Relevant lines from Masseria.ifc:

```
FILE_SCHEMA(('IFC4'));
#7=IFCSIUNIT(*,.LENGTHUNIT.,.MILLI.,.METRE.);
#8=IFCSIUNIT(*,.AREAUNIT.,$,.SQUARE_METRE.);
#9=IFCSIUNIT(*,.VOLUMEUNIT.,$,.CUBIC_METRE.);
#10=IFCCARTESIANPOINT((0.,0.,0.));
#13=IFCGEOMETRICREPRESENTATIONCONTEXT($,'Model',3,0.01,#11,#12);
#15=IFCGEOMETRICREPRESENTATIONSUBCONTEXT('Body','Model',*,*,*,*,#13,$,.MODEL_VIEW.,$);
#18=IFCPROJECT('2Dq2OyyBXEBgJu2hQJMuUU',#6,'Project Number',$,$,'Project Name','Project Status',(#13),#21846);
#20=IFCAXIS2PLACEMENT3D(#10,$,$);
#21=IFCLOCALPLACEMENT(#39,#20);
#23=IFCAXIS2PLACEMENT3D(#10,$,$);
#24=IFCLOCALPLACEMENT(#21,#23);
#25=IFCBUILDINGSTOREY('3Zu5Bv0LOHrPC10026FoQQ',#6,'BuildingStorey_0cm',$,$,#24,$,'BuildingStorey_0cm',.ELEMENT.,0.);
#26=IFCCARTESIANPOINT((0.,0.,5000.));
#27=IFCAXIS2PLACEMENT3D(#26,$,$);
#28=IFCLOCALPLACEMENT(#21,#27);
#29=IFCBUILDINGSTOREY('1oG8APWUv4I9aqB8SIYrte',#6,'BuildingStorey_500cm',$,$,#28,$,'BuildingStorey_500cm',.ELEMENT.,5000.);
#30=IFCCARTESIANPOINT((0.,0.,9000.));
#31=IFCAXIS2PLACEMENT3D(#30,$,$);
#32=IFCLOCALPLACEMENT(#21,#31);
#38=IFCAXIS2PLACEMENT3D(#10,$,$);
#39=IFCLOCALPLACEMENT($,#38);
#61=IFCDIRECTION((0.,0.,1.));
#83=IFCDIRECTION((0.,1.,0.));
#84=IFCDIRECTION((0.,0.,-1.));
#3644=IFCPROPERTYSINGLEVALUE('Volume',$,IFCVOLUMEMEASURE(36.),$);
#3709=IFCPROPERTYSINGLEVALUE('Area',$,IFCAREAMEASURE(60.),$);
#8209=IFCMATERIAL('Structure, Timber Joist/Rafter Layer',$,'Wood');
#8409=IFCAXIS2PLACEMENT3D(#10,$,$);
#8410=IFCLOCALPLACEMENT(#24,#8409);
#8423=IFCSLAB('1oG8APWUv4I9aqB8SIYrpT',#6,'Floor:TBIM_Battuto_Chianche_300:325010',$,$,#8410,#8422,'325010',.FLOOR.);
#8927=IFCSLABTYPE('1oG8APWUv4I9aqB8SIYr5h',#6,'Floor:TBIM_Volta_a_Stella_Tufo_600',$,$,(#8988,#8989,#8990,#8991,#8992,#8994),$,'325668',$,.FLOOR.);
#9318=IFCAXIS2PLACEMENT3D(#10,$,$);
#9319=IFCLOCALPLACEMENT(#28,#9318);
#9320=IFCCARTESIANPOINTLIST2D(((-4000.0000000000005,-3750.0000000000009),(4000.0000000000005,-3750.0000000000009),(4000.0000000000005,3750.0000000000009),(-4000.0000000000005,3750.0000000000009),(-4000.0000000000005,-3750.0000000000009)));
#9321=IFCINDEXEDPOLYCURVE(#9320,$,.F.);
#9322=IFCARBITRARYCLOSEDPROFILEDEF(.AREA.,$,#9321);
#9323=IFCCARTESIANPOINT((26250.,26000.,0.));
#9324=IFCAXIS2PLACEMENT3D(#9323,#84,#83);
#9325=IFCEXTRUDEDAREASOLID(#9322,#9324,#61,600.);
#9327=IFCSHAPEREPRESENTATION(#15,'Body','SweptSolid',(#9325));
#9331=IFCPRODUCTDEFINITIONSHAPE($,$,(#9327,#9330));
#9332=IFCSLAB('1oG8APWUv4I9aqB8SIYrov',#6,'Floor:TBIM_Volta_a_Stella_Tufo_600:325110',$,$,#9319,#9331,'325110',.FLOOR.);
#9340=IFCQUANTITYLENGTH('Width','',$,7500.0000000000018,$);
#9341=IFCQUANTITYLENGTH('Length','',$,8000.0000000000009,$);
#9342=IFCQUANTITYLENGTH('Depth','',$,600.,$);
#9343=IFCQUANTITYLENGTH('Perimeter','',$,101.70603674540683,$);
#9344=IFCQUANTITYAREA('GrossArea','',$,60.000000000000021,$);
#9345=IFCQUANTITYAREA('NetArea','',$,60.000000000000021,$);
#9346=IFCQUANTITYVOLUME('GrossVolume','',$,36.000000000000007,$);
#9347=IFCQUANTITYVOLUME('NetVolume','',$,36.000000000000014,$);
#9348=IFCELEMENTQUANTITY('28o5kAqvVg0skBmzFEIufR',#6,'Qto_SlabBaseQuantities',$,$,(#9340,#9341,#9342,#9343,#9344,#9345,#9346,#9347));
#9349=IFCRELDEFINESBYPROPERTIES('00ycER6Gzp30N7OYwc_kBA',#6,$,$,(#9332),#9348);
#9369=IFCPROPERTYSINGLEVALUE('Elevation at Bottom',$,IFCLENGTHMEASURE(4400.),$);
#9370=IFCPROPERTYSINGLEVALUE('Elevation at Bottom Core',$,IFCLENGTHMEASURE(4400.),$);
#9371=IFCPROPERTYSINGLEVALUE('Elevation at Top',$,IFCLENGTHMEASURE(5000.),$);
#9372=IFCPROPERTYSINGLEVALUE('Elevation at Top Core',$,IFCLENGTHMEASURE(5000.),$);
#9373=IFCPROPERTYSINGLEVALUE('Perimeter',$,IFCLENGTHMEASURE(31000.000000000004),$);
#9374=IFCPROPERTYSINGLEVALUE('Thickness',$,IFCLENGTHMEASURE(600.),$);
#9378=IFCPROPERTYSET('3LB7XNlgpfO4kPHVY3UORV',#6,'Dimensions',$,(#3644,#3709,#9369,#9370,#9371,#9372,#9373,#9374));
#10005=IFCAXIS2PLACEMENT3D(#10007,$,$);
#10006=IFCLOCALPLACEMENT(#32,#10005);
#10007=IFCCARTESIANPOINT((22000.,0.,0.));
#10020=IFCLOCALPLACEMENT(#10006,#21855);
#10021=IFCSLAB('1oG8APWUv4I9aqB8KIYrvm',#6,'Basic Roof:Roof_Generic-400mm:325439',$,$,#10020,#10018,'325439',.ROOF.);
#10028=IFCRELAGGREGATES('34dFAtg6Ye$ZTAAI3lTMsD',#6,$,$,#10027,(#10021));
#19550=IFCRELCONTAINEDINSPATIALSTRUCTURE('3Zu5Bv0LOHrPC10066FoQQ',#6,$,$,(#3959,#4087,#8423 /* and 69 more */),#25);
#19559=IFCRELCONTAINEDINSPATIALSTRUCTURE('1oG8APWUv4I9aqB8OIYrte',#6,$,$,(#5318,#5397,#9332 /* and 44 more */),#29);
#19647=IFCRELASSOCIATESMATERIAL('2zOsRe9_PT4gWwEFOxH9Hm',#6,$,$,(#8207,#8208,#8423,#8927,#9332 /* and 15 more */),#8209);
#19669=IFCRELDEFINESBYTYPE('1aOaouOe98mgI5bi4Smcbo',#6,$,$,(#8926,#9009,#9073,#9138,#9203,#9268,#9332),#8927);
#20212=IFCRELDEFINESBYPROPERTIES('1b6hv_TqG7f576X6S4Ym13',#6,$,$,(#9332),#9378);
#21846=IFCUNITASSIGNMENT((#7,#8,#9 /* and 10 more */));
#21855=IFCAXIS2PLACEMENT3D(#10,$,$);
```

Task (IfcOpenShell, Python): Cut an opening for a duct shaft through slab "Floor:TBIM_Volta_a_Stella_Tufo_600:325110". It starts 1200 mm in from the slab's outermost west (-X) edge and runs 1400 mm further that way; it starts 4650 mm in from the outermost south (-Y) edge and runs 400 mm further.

```python
import numpy as np
import ifcopenshell
import ifcopenshell.api.feature
import ifcopenshell.api.geometry
import ifcopenshell.api.pset
import ifcopenshell.api.root
import ifcopenshell.geom
import ifcopenshell.util.element
import ifcopenshell.util.placement
import ifcopenshell.util.representation
import ifcopenshell.util.shape
import ifcopenshell.util.unit

model = ifcopenshell.open("Masseria.ifc")
unit_scale = ifcopenshell.util.unit.calculate_unit_scale(model)
area_scale = ifcopenshell.util.unit.calculate_unit_scale(model, "AREAUNIT")
volume_scale = ifcopenshell.util.unit.calculate_unit_scale(model, "VOLUMEUNIT")
settings = ifcopenshell.geom.settings()


def volume(element):
    """Net volume in cubic metres, openings subtracted."""
    shape = ifcopenshell.geom.create_shape(settings, element)
    return ifcopenshell.util.shape.get_volume(shape.geometry)


slab = model.by_id(9332)
before = volume(slab)

# Extent in the slab's own axes, in metres. The edges named are its -X and -Y sides.
slab_shape = ifcopenshell.geom.create_shape(settings, slab)
vertices = ifcopenshell.util.shape.get_vertices(slab_shape.geometry)
x_min, y_min, bottom = vertices.min(axis=0)
top = vertices[:, 2].max()

opening = ifcopenshell.api.root.create_entity(model, ifc_class="IfcOpeningElement", name="Duct shaft opening", predefined_type="OPENING")
context = ifcopenshell.util.representation.get_context(model, "Model", "Body", "MODEL_VIEW")
width, depth = 1.4, 0.4
outline = [(0.0, 0.0), (width, 0.0), (width, depth), (0.0, depth), (0.0, 0.0)]
# Overshoot both faces by 50 mm so the cut is clean.
shape = ifcopenshell.api.geometry.add_slab_representation(
    model, context=context, depth=top - bottom + 0.1, polyline=outline
)
ifcopenshell.api.geometry.assign_representation(model, product=opening, representation=shape)

matrix = ifcopenshell.util.placement.get_local_placement(slab.ObjectPlacement)
matrix[:, 3] = matrix @ np.append(np.array([x_min + 1.2, y_min + 4.65, bottom - 0.05]) / unit_scale, 1.0)
ifcopenshell.api.geometry.edit_object_placement(model, product=opening, matrix=matrix, is_si=False)
ifcopenshell.api.feature.add_feature(model, feature=opening, element=slab)

after = volume(slab)

# Update the slab's stored quantities.
qto = model.by_id(ifcopenshell.util.element.get_pset(slab, "Qto_SlabBaseQuantities", should_inherit=False)["id"])
ifcopenshell.api.pset.edit_qto(model, qto=qto, properties={
    "NetArea": after / (top - bottom) / area_scale,
    "NetVolume": after / volume_scale,
})
pset = model.by_id(ifcopenshell.util.element.get_pset(slab, "Dimensions", should_inherit=False)["id"])
ifcopenshell.api.pset.edit_pset(model, pset=pset, properties={
    "Volume": model.create_entity("IfcVolumeMeasure", after / volume_scale),
    "Area": model.create_entity("IfcAreaMeasure", after / (top - bottom) / area_scale),
})

print(f"slab volume {before:.3f} -> {after:.3f} m3")

model.write("Masseria_rev.ifc")
```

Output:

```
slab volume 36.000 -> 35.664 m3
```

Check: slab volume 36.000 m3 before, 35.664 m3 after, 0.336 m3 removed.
